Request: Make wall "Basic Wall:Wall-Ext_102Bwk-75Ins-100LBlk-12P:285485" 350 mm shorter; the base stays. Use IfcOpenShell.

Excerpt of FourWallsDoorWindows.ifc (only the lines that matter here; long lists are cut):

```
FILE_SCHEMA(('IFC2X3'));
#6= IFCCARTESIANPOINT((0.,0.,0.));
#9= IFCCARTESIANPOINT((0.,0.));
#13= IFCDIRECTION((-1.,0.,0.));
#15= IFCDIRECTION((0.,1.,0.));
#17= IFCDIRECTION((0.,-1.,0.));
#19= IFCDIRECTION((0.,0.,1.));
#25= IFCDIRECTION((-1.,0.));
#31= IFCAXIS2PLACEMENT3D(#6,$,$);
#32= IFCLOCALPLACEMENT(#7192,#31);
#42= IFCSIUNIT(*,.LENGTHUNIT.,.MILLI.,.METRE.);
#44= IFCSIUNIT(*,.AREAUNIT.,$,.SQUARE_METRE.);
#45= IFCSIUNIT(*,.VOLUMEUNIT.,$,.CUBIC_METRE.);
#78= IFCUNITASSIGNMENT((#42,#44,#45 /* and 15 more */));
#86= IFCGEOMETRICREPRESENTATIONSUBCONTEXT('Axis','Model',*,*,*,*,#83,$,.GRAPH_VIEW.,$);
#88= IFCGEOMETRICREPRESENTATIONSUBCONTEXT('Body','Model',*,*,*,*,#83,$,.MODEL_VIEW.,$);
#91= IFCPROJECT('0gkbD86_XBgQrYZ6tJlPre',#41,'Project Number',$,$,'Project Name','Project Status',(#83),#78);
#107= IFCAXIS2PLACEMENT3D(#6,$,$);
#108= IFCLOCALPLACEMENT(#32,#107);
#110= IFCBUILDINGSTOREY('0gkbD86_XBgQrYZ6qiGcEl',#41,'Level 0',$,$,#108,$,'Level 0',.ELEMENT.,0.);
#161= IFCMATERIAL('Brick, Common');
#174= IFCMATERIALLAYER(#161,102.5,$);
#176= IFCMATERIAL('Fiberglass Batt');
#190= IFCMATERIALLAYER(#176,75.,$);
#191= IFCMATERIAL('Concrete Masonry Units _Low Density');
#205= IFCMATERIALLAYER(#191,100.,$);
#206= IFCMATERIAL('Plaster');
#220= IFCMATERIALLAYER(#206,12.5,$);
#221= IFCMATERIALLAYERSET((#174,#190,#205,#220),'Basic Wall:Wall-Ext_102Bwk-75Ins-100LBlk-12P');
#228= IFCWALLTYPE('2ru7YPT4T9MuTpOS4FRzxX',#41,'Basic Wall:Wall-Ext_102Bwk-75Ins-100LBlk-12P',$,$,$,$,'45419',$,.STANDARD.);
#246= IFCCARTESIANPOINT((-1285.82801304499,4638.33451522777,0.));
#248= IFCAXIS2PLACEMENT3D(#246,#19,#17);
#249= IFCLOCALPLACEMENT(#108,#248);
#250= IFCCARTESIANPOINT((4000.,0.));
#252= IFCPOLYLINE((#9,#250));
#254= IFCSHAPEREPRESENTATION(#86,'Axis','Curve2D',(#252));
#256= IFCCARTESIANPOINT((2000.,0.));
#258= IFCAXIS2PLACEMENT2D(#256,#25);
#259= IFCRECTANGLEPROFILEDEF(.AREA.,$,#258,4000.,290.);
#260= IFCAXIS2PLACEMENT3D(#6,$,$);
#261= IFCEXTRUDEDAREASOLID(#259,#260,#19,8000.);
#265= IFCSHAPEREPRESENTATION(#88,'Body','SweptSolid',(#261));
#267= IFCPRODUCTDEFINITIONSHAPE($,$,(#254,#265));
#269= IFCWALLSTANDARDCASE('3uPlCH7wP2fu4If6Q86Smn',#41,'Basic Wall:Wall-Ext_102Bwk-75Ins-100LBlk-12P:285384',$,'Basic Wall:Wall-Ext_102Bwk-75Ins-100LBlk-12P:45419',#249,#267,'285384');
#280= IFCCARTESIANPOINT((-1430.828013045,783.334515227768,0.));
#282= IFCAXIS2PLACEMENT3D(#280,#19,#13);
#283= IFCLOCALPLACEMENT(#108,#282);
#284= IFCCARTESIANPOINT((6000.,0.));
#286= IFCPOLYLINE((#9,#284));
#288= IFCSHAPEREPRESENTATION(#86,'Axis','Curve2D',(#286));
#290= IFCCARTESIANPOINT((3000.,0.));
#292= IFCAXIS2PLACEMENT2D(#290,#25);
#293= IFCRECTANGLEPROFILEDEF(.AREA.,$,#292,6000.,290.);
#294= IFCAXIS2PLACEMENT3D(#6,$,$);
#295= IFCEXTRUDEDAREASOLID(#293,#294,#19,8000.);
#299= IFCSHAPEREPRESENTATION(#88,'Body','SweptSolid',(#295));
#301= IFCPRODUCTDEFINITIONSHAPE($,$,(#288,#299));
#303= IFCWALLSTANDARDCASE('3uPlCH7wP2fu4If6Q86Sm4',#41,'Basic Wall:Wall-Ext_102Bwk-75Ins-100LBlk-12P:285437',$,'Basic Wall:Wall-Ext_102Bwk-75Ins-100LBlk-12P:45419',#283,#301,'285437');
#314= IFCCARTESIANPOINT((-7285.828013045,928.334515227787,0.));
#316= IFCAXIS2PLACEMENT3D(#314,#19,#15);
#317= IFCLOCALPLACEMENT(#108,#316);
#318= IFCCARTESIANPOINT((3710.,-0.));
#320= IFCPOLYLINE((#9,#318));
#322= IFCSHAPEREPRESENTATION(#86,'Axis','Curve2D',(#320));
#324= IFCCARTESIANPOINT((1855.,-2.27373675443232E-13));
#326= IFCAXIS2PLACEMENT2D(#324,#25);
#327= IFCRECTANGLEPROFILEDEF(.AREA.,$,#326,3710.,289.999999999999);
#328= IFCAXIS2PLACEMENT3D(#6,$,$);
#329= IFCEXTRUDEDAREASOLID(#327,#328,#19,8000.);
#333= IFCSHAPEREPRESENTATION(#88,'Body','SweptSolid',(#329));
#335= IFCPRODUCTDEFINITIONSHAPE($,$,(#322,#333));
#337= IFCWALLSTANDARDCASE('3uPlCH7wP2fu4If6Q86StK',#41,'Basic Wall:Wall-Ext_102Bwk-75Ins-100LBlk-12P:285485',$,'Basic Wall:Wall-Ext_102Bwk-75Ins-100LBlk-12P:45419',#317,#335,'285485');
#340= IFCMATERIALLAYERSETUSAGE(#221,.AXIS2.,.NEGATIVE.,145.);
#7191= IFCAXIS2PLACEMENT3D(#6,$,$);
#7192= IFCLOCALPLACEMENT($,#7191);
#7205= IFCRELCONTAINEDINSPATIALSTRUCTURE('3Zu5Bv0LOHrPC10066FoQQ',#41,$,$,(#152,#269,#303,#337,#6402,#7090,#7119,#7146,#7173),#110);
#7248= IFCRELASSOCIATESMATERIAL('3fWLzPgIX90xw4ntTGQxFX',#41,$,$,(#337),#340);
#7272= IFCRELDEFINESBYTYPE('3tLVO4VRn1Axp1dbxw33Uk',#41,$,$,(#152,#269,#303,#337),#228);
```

```python
import ifcopenshell
import ifcopenshell.geom
import ifcopenshell.util.representation
import ifcopenshell.util.shape

model = ifcopenshell.open("FourWallsDoorWindows.ifc")
settings = ifcopenshell.geom.settings()


def volume(element):
    """Net volume in cubic metres, openings subtracted."""
    shape = ifcopenshell.geom.create_shape(settings, element)
    return ifcopenshell.util.shape.get_volume(shape.geometry)


wall = model.by_id(337)
before = volume(wall)

body = ifcopenshell.util.representation.get_representation(wall, "Model", "Body")
solid = body.Items[0]
old_height = solid.Depth
solid.Depth -= 350.0
after = volume(wall)

print(f"height {old_height:g} -> {solid.Depth:g}, volume {before:.3f} -> {after:.3f} m3")

model.write("FourWallsDoorWindows_updated.ifc")
```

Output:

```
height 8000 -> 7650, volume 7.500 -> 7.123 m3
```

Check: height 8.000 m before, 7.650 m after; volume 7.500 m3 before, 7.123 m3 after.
